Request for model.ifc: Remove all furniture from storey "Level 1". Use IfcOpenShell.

First a look at what the model holds.

```python
import ifcopenshell
import ifcopenshell.util.element

model = ifcopenshell.open("model.ifc")
print(model.schema)
storey = next(s for s in model.by_type("IfcBuildingStorey") if s.Name == "Level 1")
furniture = [e for e in ifcopenshell.util.element.get_decomposition(storey) if e.is_a("IfcFurnishingElement")]
seen = {}
for e in furniture:
    element_type = ifcopenshell.util.element.get_type(e)
    name = element_type.Name if element_type not in (None, e) else None
    seen[name] = seen.get(name, 0) + 1
for name, count in sorted(seen.items(), key=str):
    print(count, "x", name)
```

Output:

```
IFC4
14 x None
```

```python
import ifcopenshell
import ifcopenshell.api.root
import ifcopenshell.util.element

model = ifcopenshell.open("model.ifc")

storey = next(s for s in model.by_type("IfcBuildingStorey") if s.Name == "Level 1")
furniture = [e for e in ifcopenshell.util.element.get_decomposition(storey) if e.is_a("IfcFurnishingElement")]

for e in furniture:
    ifcopenshell.api.root.remove_product(model, product=e)
print(len(furniture), "removed")

model.write("model_updated.ifc")
```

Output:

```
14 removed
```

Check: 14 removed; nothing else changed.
